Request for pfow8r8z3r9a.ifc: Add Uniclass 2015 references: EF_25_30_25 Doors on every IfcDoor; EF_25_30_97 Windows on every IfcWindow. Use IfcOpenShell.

First a look at what the model holds.

```python
import ifcopenshell

model = ifcopenshell.open("pfow8r8z3r9a.ifc")
print(model.schema)
print("classifications:", [c.Name for c in model.by_type("IfcClassification")])
for ifc_class in ("IfcDoor", "IfcRoof", "IfcStair", "IfcWall", "IfcWindow"):
    print(ifc_class, len(model.by_type(ifc_class)))
```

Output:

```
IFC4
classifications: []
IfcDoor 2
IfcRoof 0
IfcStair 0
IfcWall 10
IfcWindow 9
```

```python
import ifcopenshell
import ifcopenshell.api.classification

model = ifcopenshell.open("pfow8r8z3r9a.ifc")

system = ifcopenshell.api.classification.add_classification(model, classification="Uniclass 2015")

codes = {
    "IfcDoor": ("EF_25_30_25", "Doors"),
    "IfcWindow": ("EF_25_30_97", "Windows"),
}
for ifc_class, (code, name) in codes.items():
    products = model.by_type(ifc_class)
    ifcopenshell.api.classification.add_reference(
        model, products=products, classification=system, identification=code, name=name
    )
    print(code, len(products))

model.write("pfow8r8z3r9a_rev.ifc")
```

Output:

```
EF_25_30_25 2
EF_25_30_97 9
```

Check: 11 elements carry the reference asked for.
